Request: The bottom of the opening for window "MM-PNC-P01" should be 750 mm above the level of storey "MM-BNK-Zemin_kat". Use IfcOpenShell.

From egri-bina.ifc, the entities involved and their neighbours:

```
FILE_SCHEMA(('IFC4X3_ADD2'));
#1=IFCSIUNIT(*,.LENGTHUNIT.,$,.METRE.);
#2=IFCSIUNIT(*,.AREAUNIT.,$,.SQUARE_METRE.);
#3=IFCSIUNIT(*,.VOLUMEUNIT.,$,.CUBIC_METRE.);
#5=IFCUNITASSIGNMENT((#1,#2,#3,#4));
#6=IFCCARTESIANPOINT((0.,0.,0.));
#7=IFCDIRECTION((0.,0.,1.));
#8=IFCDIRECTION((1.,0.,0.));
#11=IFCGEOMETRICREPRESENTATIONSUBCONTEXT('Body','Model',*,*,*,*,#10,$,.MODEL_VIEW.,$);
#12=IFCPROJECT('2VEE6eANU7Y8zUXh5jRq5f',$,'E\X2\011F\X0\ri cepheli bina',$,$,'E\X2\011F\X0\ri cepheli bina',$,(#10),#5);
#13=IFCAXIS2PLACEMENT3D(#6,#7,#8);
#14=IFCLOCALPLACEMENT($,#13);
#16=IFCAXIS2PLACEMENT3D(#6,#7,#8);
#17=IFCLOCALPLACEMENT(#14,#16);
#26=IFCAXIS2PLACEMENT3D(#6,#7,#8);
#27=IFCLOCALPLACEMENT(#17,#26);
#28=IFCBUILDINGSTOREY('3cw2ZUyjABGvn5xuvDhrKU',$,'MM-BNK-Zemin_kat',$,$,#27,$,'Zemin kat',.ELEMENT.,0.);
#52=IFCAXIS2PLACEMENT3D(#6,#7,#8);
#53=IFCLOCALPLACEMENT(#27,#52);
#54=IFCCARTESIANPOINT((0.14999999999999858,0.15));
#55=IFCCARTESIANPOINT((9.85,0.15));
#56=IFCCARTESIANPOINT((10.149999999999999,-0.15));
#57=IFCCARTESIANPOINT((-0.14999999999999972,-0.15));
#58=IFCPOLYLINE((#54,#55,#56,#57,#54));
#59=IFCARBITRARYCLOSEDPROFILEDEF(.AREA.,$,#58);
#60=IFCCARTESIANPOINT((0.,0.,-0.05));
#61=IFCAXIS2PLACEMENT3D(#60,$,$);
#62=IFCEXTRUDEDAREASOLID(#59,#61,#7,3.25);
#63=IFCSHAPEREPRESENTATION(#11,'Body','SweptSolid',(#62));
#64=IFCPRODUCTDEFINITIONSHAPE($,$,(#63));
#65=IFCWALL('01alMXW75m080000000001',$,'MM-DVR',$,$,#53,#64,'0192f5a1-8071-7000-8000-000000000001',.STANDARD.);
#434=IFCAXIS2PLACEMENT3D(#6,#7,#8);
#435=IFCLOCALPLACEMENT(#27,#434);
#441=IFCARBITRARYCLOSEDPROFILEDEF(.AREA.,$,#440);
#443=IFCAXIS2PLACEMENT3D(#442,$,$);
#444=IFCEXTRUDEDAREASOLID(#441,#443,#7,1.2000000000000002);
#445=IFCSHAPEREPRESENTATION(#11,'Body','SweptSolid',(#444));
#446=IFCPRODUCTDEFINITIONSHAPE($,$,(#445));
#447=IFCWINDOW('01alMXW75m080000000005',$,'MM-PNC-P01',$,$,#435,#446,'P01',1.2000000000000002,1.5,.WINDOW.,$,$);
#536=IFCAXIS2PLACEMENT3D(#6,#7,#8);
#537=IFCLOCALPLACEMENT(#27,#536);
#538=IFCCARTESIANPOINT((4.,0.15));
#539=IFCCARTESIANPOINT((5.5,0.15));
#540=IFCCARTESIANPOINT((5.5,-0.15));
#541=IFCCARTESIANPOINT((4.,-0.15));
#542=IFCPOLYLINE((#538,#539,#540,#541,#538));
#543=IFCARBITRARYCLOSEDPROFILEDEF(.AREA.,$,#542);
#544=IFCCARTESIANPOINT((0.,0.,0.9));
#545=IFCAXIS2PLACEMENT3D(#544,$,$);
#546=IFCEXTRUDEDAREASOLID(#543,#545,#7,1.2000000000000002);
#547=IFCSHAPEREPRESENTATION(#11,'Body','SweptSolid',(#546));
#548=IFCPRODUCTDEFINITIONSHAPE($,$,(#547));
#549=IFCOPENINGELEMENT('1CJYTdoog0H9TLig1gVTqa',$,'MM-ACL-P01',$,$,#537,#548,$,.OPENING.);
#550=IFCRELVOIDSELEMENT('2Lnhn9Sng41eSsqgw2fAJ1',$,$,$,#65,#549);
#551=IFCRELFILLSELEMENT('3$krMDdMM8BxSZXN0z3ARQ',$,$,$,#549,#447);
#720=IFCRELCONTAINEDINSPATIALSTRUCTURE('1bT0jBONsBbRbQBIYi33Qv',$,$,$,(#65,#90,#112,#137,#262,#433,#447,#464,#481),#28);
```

```python
import numpy as np
import ifcopenshell
import ifcopenshell.api.geometry
import ifcopenshell.geom
import ifcopenshell.util.element
import ifcopenshell.util.placement
import ifcopenshell.util.shape
import ifcopenshell.util.unit

model = ifcopenshell.open("egri-bina.ifc")
unit_scale = ifcopenshell.util.unit.calculate_unit_scale(model)

window = model.by_guid("01alMXW75m080000000005")
opening = window.FillsVoids[0].RelatingOpeningElement
storey = ifcopenshell.util.element.get_container(window, ifc_class="IfcBuildingStorey")
level = ifcopenshell.util.placement.get_local_placement(storey.ObjectPlacement)[2, 3]

# The opening's origin need not be at the sill, so measure its lowest point.
shape = ifcopenshell.geom.create_shape(ifcopenshell.geom.settings(), opening)
bottom = ifcopenshell.util.shape.get_shape_bottom_elevation(shape, shape.geometry) / unit_scale
dz = level + 0.75 - bottom

shift = np.array([0.0, 0.0, dz])
# The window is not placed relative to its opening, so move both.
for product in (opening, window):
    matrix = ifcopenshell.util.placement.get_local_placement(product.ObjectPlacement)
    matrix[:3, 3] += shift
    ifcopenshell.api.geometry.edit_object_placement(model, product=product, matrix=matrix, is_si=False)

print(f"moved by {dz * unit_scale:+.3f} m")

model.write("egri-bina_rev.ifc")
```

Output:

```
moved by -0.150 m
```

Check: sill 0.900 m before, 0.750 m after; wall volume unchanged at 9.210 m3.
